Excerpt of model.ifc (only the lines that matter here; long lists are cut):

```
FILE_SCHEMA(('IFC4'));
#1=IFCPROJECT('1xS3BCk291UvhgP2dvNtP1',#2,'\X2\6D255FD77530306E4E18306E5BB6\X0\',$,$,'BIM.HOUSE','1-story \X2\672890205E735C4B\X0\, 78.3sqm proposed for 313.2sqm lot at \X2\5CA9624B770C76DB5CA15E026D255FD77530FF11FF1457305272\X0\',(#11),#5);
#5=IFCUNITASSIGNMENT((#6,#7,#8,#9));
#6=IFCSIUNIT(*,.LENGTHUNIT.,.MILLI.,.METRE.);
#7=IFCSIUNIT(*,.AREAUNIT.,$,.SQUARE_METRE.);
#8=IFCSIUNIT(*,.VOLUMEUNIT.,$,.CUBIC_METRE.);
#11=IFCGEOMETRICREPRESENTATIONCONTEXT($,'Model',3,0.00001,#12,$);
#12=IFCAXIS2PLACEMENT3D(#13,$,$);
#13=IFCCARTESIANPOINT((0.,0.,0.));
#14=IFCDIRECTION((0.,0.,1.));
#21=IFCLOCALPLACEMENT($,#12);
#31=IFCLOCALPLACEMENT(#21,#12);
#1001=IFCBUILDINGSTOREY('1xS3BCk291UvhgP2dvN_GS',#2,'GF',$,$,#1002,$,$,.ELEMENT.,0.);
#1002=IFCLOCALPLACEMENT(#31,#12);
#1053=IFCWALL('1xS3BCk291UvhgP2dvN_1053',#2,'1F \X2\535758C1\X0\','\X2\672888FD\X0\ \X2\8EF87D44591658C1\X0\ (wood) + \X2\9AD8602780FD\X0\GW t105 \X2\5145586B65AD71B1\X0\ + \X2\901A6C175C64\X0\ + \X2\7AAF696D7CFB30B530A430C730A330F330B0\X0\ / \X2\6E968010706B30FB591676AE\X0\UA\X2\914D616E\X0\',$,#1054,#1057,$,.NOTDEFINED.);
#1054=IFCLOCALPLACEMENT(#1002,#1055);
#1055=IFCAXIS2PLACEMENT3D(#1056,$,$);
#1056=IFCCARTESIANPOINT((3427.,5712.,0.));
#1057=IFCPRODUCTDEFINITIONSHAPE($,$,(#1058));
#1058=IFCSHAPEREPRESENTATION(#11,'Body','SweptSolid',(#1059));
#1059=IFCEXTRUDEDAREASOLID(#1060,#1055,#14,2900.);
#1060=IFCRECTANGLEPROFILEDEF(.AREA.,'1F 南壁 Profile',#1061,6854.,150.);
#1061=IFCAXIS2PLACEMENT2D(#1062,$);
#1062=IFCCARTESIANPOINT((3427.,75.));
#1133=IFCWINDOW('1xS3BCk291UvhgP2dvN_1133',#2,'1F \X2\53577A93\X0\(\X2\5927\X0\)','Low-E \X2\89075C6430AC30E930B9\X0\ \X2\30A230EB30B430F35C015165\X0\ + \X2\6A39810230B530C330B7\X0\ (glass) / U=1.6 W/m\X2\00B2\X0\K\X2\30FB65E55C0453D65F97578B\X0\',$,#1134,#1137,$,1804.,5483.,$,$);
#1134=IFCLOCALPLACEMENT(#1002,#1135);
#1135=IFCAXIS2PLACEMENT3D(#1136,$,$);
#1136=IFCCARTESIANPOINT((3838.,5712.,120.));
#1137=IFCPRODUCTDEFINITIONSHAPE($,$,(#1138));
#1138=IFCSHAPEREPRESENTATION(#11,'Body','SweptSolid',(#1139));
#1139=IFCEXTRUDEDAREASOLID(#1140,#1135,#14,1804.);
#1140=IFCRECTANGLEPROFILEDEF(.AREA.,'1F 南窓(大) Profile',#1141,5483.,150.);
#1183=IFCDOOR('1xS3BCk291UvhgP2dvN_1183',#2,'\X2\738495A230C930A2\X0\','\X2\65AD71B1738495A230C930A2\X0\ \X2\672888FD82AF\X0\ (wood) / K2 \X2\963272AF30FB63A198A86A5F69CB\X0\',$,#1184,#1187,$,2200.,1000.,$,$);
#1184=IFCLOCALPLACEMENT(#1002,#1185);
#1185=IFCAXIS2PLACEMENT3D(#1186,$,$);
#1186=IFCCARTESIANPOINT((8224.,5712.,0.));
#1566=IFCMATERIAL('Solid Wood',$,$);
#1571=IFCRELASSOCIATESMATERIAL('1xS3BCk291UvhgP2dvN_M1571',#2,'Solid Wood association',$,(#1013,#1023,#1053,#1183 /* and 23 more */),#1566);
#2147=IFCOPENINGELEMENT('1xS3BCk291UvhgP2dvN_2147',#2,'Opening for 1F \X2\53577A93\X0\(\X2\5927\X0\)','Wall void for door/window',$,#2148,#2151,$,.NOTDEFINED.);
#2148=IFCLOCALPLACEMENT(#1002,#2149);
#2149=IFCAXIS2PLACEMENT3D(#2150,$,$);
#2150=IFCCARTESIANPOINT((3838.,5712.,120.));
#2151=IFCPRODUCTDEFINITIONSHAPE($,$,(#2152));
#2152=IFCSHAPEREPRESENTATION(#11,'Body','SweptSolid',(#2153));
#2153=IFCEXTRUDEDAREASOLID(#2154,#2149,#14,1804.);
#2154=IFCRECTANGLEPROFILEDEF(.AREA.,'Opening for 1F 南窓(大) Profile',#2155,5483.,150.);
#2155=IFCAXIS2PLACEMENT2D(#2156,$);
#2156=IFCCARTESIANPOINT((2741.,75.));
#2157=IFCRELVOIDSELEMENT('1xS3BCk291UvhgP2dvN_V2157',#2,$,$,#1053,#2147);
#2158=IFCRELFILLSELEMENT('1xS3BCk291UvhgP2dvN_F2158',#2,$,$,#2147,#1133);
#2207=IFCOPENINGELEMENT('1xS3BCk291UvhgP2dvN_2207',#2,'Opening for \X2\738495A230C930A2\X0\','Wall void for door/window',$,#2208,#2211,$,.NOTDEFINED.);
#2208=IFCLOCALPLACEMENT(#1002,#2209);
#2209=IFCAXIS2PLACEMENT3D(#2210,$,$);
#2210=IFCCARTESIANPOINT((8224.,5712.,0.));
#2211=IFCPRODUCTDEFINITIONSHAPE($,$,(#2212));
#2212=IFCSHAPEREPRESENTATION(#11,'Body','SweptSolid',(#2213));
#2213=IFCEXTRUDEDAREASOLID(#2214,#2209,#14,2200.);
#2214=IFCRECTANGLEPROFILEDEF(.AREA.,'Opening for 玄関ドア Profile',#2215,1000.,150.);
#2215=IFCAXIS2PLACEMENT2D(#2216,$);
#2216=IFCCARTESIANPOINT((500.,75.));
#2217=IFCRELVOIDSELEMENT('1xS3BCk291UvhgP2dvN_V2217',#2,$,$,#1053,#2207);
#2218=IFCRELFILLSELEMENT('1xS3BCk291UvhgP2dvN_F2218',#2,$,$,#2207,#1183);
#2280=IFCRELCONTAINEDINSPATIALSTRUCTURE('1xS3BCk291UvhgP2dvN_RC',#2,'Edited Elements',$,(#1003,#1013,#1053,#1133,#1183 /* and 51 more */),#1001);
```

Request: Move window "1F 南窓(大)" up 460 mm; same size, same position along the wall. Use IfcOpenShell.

```python
import numpy as np
import ifcopenshell
import ifcopenshell.api.geometry
import ifcopenshell.util.placement
import ifcopenshell.util.unit

model = ifcopenshell.open("model.ifc")
unit_scale = ifcopenshell.util.unit.calculate_unit_scale(model)

window = model.by_guid("1xS3BCk291UvhgP2dvN_1133")
opening = window.FillsVoids[0].RelatingOpeningElement
dz = 0.46 / unit_scale

shift = np.array([0.0, 0.0, dz])
# The window is not placed relative to its opening, so move both.
for product in (opening, window):
    matrix = ifcopenshell.util.placement.get_local_placement(product.ObjectPlacement)
    matrix[:3, 3] += shift
    ifcopenshell.api.geometry.edit_object_placement(model, product=product, matrix=matrix, is_si=False)

print(f"moved by {dz * unit_scale:+.3f} m")

model.write("model-out.ifc")
```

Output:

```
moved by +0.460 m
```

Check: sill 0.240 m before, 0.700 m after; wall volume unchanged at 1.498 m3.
